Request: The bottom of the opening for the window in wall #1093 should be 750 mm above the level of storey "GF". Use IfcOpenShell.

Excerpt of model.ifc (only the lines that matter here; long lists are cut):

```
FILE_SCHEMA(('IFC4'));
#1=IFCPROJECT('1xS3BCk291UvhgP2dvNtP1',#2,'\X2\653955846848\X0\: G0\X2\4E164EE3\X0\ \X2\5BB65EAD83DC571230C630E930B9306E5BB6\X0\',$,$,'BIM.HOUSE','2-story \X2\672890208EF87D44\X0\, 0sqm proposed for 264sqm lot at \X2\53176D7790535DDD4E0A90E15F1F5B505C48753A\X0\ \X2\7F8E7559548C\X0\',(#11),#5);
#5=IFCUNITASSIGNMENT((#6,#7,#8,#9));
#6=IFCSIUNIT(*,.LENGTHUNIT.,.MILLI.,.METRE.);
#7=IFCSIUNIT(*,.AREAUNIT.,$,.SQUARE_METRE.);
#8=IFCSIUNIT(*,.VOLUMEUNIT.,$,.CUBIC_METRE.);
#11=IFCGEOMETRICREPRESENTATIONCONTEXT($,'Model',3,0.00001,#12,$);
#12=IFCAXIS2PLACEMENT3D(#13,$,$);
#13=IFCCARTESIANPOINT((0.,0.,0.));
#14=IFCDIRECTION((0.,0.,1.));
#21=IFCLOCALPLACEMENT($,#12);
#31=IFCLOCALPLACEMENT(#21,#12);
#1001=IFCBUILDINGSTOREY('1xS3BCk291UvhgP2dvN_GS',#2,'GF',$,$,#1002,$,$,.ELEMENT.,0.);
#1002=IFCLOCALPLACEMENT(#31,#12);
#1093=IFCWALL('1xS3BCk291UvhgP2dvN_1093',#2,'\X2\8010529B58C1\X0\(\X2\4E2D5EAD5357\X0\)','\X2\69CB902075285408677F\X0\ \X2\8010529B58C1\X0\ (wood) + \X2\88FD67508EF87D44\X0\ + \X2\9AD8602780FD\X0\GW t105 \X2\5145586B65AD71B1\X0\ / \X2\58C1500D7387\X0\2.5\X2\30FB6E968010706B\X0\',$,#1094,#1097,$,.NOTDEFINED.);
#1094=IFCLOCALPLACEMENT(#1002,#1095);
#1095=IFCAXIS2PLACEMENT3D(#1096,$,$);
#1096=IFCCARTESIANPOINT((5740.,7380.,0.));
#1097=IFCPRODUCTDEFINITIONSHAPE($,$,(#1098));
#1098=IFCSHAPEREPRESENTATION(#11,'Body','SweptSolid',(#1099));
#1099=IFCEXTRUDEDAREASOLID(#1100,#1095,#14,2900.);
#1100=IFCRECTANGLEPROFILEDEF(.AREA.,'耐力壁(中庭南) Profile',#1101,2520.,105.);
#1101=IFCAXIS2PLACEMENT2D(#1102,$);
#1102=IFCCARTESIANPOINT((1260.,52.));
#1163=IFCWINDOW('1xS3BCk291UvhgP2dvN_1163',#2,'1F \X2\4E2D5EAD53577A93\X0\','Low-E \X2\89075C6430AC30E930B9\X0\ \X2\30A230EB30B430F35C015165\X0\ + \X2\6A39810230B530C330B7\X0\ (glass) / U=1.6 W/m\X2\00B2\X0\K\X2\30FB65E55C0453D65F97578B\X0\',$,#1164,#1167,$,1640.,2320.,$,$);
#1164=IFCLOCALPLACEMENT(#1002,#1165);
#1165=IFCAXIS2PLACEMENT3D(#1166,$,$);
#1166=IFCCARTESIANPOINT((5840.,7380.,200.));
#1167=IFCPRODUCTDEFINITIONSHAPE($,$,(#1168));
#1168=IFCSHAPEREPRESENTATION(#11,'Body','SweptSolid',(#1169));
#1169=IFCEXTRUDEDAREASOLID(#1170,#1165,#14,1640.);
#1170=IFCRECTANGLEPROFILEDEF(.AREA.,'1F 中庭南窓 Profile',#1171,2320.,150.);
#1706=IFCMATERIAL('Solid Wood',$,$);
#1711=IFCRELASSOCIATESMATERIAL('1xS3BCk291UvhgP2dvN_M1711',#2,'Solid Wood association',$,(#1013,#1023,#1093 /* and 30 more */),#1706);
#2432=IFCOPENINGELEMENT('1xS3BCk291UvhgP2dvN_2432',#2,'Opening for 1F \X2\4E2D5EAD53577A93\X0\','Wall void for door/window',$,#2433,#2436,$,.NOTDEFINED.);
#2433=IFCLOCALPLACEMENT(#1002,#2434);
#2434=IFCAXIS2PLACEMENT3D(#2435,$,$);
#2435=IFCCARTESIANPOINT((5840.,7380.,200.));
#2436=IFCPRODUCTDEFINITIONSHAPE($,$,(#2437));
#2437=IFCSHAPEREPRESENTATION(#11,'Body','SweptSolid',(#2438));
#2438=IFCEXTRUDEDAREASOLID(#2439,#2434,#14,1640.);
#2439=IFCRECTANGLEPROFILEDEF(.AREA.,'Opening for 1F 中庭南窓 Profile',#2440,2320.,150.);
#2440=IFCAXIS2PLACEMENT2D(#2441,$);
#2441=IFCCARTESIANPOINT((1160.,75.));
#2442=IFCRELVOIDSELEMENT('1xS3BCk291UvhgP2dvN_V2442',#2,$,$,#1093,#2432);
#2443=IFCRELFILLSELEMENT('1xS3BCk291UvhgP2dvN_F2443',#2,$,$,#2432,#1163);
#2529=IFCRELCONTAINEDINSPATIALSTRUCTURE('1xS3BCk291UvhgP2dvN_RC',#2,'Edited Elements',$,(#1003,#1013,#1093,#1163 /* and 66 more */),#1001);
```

```python
import numpy as np
import ifcopenshell
import ifcopenshell.api.geometry
import ifcopenshell.geom
import ifcopenshell.util.element
import ifcopenshell.util.placement
import ifcopenshell.util.shape
import ifcopenshell.util.unit

model = ifcopenshell.open("model.ifc")
unit_scale = ifcopenshell.util.unit.calculate_unit_scale(model)

window = model.by_id(1163)
opening = window.FillsVoids[0].RelatingOpeningElement
storey = ifcopenshell.util.element.get_container(window, ifc_class="IfcBuildingStorey")
level = ifcopenshell.util.placement.get_local_placement(storey.ObjectPlacement)[2, 3]

# The opening's origin need not be at the sill, so measure its lowest point.
shape = ifcopenshell.geom.create_shape(ifcopenshell.geom.settings(), opening)
bottom = ifcopenshell.util.shape.get_shape_bottom_elevation(shape, shape.geometry) / unit_scale
dz = level + 0.75 / unit_scale - bottom

shift = np.array([0.0, 0.0, dz])
# The window is not placed relative to its opening, so move both.
for product in (opening, window):
    matrix = ifcopenshell.util.placement.get_local_placement(product.ObjectPlacement)
    matrix[:3, 3] += shift
    ifcopenshell.api.geometry.edit_object_placement(model, product=product, matrix=matrix, is_si=False)

print(f"moved by {dz * unit_scale:+.3f} m")

model.write("model_edited.ifc")
```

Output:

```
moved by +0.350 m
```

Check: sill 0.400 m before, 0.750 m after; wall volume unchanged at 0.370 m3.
